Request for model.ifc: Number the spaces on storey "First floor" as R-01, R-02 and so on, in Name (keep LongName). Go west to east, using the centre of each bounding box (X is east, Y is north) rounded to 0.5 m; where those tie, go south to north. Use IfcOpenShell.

First a look at what the model holds.

```python
import ifcopenshell
import ifcopenshell.util.element
import ifcopenshell.util.placement

model = ifcopenshell.open("model.ifc")
print(model.schema)
storey = next(s for s in model.by_type("IfcBuildingStorey") if s.Name == "First floor")
spaces = [e for e in ifcopenshell.util.element.get_decomposition(storey) if e.is_a("IfcSpace")]
for e in sorted(spaces, key=lambda e: e.id()):
    origin = ifcopenshell.util.placement.get_local_placement(e.ObjectPlacement)[:3, 3]
    print(e.id(), e.Name, e.LongName, origin.round(2) + 0.0, sep=" | ")
```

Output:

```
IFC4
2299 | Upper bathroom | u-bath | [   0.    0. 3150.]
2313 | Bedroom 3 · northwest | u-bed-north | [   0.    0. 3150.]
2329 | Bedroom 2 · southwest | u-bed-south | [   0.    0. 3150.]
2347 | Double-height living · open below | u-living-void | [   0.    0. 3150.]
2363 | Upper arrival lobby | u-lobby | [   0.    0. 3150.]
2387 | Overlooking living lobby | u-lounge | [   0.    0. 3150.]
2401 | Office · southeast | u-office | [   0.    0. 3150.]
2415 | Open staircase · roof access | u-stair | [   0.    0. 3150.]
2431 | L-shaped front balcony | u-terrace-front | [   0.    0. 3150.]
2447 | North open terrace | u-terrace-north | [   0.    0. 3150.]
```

```python
import ifcopenshell
import ifcopenshell.geom
import ifcopenshell.util.element
import ifcopenshell.util.shape

model = ifcopenshell.open("model.ifc")
settings = ifcopenshell.geom.settings()
settings.set("use-world-coords", True)


def centre(element):
    shape = ifcopenshell.geom.create_shape(settings, element)
    return ifcopenshell.util.shape.get_bbox_centroid(shape.geometry)


storey = next(s for s in model.by_type("IfcBuildingStorey") if s.Name == "First floor")
spaces = [e for e in ifcopenshell.util.element.get_decomposition(storey) if e.is_a("IfcSpace")]

# Insertion points can sit at a corner or the storey origin, so sort by the geometry (in metres).
centres = {e: centre(e) for e in spaces}
spaces.sort(key=lambda e: (round(centres[e][0] / 0.5), centres[e][1]))

for i, e in enumerate(spaces, start=1):
    number = f"R-{i:02d}"
    e.Name = number
    print(e.id(), number)

model.write("model_updated.ifc")
```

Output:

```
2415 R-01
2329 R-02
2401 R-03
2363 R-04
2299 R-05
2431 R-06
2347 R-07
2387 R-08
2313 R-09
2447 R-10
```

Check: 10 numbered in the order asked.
